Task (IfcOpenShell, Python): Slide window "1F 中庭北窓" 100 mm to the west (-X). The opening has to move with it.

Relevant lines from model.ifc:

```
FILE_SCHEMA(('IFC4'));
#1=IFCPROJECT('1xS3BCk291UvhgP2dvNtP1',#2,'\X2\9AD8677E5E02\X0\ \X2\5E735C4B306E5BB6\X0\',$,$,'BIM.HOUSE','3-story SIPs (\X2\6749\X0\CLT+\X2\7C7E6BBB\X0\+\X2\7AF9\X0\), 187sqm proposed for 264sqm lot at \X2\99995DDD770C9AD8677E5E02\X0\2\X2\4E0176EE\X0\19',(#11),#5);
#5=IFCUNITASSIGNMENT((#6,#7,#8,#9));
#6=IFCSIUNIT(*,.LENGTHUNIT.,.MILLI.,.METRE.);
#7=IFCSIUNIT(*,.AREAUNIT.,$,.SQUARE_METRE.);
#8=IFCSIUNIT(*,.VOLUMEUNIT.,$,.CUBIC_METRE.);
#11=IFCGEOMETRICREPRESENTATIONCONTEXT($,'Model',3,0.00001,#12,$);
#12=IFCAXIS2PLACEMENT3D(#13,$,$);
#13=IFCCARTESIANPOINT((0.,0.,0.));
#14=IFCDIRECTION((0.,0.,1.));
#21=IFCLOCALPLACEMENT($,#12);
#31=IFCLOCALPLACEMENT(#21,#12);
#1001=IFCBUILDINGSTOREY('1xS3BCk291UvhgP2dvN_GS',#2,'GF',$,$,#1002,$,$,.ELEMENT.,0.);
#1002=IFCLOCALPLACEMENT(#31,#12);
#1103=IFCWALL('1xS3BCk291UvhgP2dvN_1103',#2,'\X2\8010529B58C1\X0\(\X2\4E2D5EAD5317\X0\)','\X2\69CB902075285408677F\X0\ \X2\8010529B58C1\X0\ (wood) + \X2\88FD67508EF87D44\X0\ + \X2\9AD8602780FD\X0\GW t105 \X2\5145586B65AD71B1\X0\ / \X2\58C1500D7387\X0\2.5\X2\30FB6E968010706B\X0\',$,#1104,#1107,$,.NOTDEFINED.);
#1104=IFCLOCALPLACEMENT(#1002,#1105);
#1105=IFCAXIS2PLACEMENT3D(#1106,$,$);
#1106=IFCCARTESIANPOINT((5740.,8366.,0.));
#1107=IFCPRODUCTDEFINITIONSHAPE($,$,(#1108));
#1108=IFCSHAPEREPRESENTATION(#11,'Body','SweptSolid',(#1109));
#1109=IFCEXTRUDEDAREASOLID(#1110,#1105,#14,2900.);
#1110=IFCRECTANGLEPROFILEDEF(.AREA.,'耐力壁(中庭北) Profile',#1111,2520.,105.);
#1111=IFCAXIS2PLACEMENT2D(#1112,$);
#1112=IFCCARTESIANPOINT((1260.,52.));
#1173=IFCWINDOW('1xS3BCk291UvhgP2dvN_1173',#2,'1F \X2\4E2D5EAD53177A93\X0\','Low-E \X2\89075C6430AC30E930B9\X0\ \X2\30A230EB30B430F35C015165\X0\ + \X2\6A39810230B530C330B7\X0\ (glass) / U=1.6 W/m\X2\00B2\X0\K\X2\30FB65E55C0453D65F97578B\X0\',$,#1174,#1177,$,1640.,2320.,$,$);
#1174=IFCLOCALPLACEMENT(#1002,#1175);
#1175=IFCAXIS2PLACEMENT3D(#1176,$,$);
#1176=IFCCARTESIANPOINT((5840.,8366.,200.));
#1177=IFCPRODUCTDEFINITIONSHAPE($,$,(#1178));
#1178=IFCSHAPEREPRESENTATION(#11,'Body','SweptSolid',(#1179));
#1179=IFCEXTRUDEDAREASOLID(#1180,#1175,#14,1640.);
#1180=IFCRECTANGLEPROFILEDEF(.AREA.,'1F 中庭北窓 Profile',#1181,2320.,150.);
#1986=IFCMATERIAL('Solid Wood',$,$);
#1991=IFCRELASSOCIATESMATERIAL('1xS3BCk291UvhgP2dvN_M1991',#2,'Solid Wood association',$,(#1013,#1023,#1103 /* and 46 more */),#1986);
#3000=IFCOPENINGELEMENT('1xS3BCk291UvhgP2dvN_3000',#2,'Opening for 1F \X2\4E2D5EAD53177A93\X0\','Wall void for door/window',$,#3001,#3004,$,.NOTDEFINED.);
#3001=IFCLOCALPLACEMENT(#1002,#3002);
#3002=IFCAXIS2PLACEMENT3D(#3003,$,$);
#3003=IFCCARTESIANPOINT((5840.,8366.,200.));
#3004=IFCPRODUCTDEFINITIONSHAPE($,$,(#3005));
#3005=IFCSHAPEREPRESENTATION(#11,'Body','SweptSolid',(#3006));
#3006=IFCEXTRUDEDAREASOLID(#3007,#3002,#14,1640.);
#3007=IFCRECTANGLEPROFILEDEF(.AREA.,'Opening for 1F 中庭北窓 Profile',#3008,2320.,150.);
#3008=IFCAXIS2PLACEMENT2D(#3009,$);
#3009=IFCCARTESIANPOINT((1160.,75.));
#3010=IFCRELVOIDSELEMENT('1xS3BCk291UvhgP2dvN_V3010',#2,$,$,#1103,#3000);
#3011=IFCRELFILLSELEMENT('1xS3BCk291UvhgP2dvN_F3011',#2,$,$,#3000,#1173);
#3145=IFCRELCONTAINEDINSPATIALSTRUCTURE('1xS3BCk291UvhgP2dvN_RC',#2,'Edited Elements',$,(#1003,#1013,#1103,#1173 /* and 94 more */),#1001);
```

```python
import ifcopenshell
import ifcopenshell.api.geometry
import ifcopenshell.util.placement
import ifcopenshell.util.unit

model = ifcopenshell.open("model.ifc")
unit_scale = ifcopenshell.util.unit.calculate_unit_scale(model)

window = model.by_guid("1xS3BCk291UvhgP2dvN_1173")
opening = window.FillsVoids[0].RelatingOpeningElement
wall = opening.VoidsElements[0].RelatingBuildingElement

wall_matrix = ifcopenshell.util.placement.get_local_placement(wall.ObjectPlacement)
shift = wall_matrix[:3, 0] * -0.1 / unit_scale
before = ifcopenshell.util.placement.get_local_placement(window.ObjectPlacement)[:3, 3].copy()

# The window is not placed relative to its opening, so move both.
for product in (opening, window):
    matrix = ifcopenshell.util.placement.get_local_placement(product.ObjectPlacement)
    matrix[:3, 3] += shift
    ifcopenshell.api.geometry.edit_object_placement(model, product=product, matrix=matrix, is_si=False)

after = ifcopenshell.util.placement.get_local_placement(window.ObjectPlacement)[:3, 3]
print("window moved by", (after - before).round(3) + 0.0)

model.write("model_updated.ifc")
```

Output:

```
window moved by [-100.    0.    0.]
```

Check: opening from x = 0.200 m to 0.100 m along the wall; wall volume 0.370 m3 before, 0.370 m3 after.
